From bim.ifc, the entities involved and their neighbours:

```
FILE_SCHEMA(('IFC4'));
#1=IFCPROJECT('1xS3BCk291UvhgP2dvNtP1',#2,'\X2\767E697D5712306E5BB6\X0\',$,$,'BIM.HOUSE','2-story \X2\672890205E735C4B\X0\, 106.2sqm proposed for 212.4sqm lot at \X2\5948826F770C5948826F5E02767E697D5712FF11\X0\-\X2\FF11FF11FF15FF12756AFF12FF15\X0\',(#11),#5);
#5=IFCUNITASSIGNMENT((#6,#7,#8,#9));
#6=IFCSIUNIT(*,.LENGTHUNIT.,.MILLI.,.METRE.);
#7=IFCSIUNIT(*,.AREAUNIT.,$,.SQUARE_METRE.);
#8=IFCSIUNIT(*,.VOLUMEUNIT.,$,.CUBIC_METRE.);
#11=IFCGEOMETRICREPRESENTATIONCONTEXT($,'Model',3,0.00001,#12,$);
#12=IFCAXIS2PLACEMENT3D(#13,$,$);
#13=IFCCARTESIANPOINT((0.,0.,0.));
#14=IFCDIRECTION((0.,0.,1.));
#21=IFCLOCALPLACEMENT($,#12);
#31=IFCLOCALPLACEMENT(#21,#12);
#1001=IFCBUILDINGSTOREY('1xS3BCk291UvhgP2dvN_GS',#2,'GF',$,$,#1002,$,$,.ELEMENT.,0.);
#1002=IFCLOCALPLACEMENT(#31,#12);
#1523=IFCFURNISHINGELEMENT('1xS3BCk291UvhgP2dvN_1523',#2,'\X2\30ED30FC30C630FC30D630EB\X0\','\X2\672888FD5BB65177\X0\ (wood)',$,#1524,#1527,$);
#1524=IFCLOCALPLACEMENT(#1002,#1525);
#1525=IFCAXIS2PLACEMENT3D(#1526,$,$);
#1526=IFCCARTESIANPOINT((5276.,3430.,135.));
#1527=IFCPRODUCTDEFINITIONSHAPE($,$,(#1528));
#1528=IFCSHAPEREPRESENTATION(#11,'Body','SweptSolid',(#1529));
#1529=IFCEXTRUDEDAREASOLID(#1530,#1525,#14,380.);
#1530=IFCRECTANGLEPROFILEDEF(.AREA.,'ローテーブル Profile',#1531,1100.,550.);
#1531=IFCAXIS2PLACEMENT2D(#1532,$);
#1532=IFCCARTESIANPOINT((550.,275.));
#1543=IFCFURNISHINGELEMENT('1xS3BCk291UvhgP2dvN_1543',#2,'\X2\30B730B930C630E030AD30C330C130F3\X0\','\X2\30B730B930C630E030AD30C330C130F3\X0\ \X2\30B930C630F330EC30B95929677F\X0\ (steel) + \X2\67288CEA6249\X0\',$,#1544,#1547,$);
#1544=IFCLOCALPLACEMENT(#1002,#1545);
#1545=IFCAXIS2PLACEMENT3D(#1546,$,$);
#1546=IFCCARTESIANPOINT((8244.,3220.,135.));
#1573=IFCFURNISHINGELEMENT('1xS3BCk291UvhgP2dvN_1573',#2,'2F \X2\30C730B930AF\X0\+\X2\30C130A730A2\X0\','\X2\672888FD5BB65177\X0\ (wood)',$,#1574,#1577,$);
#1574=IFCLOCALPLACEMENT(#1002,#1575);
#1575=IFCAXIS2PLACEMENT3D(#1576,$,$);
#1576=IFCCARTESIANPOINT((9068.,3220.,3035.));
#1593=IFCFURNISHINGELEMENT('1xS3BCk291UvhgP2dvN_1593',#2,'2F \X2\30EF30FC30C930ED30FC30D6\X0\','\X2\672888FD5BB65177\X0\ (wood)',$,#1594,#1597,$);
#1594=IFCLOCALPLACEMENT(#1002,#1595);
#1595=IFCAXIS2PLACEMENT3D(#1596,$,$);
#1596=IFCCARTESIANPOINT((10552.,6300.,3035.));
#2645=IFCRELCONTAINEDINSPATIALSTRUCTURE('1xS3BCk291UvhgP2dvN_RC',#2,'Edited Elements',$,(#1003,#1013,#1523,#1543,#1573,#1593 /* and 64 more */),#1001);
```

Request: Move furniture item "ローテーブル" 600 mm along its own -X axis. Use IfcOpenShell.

```python
import ifcopenshell
import ifcopenshell.api.geometry
import ifcopenshell.util.placement
import ifcopenshell.util.unit

model = ifcopenshell.open("bim.ifc")
unit_scale = ifcopenshell.util.unit.calculate_unit_scale(model)

item = model.by_guid("1xS3BCk291UvhgP2dvN_1523")
matrix = ifcopenshell.util.placement.get_local_placement(item.ObjectPlacement)
matrix[:3, 3] -= matrix[:3, 0] * 0.6 / unit_scale
ifcopenshell.api.geometry.edit_object_placement(model, product=item, matrix=matrix, is_si=False)

print(ifcopenshell.util.placement.get_local_placement(item.ObjectPlacement).round(3) + 0.0)

model.write("bim-out.ifc")
```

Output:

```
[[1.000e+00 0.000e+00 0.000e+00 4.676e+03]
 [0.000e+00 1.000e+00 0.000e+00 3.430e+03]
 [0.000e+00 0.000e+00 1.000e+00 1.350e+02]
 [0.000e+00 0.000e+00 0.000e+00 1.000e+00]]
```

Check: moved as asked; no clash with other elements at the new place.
